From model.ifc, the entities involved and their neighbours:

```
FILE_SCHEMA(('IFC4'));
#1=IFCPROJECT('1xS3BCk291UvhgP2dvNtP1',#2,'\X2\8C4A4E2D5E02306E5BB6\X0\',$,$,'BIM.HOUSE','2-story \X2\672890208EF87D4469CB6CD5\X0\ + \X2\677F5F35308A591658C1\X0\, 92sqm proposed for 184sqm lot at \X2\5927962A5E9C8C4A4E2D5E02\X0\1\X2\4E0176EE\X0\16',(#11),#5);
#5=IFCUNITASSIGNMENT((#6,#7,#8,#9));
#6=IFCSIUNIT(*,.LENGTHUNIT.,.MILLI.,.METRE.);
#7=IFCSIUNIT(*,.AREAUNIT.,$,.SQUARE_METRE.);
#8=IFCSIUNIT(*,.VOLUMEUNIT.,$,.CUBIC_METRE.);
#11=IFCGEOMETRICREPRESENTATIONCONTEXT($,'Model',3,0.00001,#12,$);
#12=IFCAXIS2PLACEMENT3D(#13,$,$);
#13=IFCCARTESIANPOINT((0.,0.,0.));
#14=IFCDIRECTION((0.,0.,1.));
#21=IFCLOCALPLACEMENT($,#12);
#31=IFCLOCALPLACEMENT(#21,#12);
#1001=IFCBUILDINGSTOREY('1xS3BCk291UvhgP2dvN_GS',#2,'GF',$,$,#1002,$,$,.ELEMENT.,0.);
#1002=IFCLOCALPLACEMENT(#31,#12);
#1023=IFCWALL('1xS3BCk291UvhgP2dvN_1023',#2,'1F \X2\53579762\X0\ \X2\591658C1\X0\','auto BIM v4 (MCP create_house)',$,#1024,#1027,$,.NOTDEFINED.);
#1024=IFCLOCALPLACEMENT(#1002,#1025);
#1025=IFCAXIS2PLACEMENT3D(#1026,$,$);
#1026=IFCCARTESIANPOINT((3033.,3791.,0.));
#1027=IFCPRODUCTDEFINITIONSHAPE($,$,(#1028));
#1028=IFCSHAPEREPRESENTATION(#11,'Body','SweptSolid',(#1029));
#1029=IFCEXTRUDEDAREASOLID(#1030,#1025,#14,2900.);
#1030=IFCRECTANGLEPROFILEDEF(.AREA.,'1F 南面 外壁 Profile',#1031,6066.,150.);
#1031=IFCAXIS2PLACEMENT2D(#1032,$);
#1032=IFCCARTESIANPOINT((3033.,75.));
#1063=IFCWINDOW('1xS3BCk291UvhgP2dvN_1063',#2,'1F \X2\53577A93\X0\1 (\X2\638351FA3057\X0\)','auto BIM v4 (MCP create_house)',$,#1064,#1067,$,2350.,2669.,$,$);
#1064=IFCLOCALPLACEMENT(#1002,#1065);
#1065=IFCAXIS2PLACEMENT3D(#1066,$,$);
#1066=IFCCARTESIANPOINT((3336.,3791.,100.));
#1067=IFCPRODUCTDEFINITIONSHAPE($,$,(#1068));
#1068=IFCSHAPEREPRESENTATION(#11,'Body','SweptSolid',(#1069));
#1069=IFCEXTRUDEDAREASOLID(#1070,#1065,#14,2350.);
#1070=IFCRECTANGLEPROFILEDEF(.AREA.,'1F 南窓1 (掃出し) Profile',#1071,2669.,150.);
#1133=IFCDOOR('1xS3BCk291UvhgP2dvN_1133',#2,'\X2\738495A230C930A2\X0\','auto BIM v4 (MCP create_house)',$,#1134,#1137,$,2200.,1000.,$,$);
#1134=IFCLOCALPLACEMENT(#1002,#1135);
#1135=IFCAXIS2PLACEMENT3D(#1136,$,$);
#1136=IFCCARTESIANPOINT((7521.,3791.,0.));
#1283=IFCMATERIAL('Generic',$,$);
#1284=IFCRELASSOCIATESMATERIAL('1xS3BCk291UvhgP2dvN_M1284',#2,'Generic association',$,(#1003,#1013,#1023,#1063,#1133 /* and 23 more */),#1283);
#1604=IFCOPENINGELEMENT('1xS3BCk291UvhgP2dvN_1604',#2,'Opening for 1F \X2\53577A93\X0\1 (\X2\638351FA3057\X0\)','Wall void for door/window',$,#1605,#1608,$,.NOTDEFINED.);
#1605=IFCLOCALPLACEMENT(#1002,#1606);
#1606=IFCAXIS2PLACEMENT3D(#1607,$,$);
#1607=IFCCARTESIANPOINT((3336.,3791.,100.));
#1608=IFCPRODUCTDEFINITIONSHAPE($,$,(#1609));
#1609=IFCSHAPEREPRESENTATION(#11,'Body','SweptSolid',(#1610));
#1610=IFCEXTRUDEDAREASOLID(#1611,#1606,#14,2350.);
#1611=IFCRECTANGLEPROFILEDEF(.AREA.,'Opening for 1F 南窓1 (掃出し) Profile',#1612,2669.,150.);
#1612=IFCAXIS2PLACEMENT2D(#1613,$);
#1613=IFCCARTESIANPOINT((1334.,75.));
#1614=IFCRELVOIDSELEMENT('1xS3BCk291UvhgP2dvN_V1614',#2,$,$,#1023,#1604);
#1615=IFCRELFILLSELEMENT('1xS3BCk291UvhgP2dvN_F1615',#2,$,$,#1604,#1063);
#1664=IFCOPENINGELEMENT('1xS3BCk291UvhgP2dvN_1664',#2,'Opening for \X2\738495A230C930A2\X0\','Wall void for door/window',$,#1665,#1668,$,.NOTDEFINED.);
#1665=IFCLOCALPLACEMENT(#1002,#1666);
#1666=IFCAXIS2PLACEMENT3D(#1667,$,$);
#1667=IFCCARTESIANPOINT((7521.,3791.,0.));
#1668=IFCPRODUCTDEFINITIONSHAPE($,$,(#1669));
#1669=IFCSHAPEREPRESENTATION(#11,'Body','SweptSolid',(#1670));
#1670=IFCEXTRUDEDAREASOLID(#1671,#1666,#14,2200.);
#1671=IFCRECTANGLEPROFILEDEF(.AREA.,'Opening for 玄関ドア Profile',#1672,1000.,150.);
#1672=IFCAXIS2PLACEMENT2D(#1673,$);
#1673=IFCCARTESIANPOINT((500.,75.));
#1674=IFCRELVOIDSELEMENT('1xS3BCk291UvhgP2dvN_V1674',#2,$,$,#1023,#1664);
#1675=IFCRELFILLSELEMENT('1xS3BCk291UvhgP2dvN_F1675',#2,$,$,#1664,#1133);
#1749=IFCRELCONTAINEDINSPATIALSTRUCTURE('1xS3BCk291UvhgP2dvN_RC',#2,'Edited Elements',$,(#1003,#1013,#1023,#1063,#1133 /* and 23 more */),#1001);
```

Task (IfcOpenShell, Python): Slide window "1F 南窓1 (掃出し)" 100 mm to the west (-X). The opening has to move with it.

```python
import ifcopenshell
import ifcopenshell.api.geometry
import ifcopenshell.util.placement

model = ifcopenshell.open("model.ifc")

window = model.by_id(1063)
opening = window.FillsVoids[0].RelatingOpeningElement
wall = opening.VoidsElements[0].RelatingBuildingElement

wall_matrix = ifcopenshell.util.placement.get_local_placement(wall.ObjectPlacement)
shift = wall_matrix[:3, 0] * -100.0
before = ifcopenshell.util.placement.get_local_placement(window.ObjectPlacement)[:3, 3].copy()

# The window is not placed relative to its opening, so move both.
for product in (opening, window):
    matrix = ifcopenshell.util.placement.get_local_placement(product.ObjectPlacement)
    matrix[:3, 3] += shift
    ifcopenshell.api.geometry.edit_object_placement(model, product=product, matrix=matrix, is_si=False)

after = ifcopenshell.util.placement.get_local_placement(window.ObjectPlacement)[:3, 3]
print("window moved by", (after - before).round(3) + 0.0)

model.write("model_rev.ifc")
```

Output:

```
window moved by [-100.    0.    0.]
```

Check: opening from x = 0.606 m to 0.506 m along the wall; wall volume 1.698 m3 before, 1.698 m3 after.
